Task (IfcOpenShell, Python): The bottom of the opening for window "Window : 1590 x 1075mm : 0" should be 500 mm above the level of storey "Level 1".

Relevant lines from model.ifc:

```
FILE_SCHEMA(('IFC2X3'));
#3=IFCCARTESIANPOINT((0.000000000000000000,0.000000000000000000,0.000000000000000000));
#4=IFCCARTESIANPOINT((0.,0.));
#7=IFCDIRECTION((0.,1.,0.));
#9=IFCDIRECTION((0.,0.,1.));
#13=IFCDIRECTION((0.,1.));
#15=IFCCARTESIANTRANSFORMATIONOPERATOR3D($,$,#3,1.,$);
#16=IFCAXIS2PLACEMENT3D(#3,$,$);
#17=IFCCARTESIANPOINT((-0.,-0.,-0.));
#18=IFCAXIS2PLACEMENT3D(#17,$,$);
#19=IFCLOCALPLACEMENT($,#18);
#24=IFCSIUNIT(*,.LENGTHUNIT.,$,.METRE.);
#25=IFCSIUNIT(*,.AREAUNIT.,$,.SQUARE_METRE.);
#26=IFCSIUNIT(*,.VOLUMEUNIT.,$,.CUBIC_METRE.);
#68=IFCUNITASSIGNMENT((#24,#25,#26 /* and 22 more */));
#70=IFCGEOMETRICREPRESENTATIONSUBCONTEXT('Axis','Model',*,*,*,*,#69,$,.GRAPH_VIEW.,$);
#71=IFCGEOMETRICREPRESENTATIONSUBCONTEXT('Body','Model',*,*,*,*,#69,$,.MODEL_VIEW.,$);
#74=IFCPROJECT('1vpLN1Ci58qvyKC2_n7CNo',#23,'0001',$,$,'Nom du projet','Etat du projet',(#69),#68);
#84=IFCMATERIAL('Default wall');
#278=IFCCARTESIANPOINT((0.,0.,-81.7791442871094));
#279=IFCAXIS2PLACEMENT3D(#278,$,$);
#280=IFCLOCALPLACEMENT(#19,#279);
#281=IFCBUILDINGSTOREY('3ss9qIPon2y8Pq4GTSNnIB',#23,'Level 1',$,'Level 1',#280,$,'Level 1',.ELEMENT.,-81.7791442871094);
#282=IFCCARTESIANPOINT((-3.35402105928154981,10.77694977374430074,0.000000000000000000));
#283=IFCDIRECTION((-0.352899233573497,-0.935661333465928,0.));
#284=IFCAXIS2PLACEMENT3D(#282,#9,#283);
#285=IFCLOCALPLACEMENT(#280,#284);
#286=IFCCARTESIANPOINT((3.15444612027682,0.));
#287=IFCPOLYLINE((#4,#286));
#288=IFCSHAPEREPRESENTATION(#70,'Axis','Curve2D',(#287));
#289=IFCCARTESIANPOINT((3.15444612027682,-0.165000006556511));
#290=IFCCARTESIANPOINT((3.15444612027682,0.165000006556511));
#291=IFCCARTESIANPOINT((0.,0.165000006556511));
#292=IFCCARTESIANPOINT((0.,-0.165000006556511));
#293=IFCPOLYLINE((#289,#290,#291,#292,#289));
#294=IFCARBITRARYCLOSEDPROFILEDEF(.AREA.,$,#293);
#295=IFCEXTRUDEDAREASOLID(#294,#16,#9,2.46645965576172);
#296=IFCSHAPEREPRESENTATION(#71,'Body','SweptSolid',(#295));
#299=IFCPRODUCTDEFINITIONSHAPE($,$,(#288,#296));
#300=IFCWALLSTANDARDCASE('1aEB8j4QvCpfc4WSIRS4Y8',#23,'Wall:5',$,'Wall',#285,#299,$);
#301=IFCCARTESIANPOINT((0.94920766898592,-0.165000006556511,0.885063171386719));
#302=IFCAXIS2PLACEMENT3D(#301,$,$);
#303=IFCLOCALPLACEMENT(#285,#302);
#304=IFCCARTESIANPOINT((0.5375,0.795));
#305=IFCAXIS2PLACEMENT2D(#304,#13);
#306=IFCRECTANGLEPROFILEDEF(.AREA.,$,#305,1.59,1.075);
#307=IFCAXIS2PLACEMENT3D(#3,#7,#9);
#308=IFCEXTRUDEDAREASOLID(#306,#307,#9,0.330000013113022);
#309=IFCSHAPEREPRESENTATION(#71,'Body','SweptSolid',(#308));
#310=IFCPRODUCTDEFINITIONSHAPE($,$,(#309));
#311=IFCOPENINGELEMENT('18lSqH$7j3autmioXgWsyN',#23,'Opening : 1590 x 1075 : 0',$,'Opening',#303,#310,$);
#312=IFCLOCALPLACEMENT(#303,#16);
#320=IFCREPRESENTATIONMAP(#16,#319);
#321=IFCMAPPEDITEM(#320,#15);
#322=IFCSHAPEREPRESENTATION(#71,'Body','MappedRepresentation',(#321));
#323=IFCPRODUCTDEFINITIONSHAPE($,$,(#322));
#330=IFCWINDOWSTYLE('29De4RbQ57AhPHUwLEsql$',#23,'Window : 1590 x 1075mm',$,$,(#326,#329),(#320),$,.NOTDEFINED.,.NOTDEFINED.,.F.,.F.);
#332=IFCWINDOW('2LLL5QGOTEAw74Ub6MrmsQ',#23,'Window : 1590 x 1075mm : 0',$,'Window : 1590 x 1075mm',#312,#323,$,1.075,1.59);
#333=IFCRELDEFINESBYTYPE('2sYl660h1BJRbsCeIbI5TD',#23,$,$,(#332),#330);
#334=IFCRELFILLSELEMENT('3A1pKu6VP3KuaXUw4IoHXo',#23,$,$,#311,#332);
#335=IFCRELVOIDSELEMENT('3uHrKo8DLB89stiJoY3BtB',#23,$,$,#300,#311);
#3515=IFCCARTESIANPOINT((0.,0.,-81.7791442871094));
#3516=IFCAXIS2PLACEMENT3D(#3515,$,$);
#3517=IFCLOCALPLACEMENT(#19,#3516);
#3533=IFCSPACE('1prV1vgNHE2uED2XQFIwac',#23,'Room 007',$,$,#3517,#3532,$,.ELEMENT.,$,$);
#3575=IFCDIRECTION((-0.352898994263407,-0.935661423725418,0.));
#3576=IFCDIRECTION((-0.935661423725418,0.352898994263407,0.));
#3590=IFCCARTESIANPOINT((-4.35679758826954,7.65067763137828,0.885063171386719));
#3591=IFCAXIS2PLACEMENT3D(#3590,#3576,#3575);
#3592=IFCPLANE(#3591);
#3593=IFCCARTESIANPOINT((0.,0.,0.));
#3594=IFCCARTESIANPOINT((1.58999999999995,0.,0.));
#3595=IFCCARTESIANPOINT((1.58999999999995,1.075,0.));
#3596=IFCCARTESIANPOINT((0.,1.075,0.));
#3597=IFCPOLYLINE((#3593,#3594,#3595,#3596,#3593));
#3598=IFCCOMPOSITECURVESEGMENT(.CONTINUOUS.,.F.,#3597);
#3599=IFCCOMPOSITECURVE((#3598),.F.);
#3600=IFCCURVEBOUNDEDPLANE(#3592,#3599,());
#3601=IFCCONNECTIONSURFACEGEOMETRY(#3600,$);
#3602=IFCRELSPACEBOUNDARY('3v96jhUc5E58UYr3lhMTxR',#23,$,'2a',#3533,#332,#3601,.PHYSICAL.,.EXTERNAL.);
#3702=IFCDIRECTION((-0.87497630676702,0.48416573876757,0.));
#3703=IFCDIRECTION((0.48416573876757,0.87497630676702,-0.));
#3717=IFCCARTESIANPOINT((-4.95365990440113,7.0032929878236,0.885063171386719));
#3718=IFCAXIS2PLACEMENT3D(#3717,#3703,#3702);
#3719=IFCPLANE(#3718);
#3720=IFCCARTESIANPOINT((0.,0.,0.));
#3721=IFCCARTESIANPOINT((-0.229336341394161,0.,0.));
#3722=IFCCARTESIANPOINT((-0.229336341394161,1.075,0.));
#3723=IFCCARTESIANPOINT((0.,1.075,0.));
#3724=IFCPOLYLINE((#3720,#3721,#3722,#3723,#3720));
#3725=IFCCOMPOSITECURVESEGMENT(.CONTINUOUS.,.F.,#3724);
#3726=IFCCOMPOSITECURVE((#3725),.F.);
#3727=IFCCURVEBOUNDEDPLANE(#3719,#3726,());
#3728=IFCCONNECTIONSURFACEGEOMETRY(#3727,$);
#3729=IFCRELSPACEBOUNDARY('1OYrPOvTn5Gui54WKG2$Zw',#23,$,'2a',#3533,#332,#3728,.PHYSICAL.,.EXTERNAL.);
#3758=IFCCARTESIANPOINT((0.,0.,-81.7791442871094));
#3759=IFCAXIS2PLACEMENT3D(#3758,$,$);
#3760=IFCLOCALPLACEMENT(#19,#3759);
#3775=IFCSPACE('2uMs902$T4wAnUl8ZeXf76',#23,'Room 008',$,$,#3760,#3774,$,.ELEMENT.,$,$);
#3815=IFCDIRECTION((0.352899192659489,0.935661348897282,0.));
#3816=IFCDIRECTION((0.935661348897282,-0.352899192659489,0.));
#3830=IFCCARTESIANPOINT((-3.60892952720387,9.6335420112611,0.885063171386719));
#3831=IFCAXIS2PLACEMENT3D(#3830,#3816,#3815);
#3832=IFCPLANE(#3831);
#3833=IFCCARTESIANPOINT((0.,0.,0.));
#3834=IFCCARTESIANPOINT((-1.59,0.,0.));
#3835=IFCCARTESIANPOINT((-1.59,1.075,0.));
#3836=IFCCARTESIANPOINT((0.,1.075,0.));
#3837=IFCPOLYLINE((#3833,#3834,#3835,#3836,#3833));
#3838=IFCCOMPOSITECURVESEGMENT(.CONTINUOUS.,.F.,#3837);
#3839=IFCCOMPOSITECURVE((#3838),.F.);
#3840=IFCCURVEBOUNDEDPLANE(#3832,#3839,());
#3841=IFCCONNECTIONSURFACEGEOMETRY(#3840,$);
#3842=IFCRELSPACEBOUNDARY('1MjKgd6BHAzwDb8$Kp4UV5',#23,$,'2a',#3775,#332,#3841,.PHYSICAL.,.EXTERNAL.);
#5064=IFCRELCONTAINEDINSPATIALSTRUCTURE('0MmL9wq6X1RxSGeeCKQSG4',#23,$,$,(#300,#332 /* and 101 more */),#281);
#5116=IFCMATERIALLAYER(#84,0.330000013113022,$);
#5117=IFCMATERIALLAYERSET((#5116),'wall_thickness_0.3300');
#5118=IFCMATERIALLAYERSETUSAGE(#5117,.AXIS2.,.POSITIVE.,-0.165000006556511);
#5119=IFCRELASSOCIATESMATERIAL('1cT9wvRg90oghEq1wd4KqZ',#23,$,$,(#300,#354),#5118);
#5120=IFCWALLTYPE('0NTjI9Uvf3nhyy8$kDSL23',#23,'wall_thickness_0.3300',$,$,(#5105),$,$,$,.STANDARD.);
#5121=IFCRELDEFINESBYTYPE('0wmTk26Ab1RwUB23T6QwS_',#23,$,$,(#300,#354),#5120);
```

```python
import numpy as np
import ifcopenshell
import ifcopenshell.api.geometry
import ifcopenshell.geom
import ifcopenshell.util.element
import ifcopenshell.util.placement
import ifcopenshell.util.shape
import ifcopenshell.util.unit

model = ifcopenshell.open("model.ifc")
unit_scale = ifcopenshell.util.unit.calculate_unit_scale(model)

window = model.by_guid("2LLL5QGOTEAw74Ub6MrmsQ")
opening = window.FillsVoids[0].RelatingOpeningElement
storey = ifcopenshell.util.element.get_container(window, ifc_class="IfcBuildingStorey")
level = ifcopenshell.util.placement.get_local_placement(storey.ObjectPlacement)[2, 3]

# The opening's origin need not be at the sill, so measure its lowest point.
shape = ifcopenshell.geom.create_shape(ifcopenshell.geom.settings(), opening)
bottom = ifcopenshell.util.shape.get_shape_bottom_elevation(shape, shape.geometry) / unit_scale
dz = level + 0.5 - bottom

shift = np.array([0.0, 0.0, dz])
# The window is placed relative to its opening, so it follows when the opening moves.
matrix = ifcopenshell.util.placement.get_local_placement(opening.ObjectPlacement)
matrix[:3, 3] += shift
ifcopenshell.api.geometry.edit_object_placement(
    model, product=opening, matrix=matrix, is_si=False, should_transform_children=True
)

# Space boundary surfaces are stored in each space's coordinates; move them too.
for rel in window.ProvidesBoundaries:
    if not rel.ConnectionGeometry:
        continue
    surface = rel.ConnectionGeometry.SurfaceOnRelatingElement.BasisSurface
    space_matrix = ifcopenshell.util.placement.get_local_placement(rel.RelatingSpace.ObjectPlacement)
    point = np.array(surface.Position.Location.Coordinates) + space_matrix[:3, :3].T @ shift
    surface.Position = model.createIfcAxis2Placement3D(
        model.createIfcCartesianPoint(point.tolist()), surface.Position.Axis, surface.Position.RefDirection
    )

print(f"moved by {dz * unit_scale:+.3f} m")

model.write("model_v2.ifc")
```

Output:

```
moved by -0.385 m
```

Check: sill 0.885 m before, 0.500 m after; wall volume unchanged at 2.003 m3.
